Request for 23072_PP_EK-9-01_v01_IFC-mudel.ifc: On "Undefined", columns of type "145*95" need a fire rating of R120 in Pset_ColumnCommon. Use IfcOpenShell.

First a look at what the model holds.

```python
import ifcopenshell
import ifcopenshell.util.element

model = ifcopenshell.open("23072_PP_EK-9-01_v01_IFC-mudel.ifc")
print(model.schema)
storey = next(s for s in model.by_type("IfcBuildingStorey") if s.Name == "Undefined")
columns = [e for e in ifcopenshell.util.element.get_decomposition(storey) if e.is_a("IfcColumn")]
seen = {}
for e in columns:
    element_type = ifcopenshell.util.element.get_type(e)
    key = (element_type.Name if element_type != e and element_type else None, ifcopenshell.util.element.get_pset(e, "Pset_ColumnCommon", "FireRating"))
    seen[key] = seen.get(key, 0) + 1
for (name, value), count in sorted(seen.items(), key=str):
    print(count, "x", name, "|", value)
```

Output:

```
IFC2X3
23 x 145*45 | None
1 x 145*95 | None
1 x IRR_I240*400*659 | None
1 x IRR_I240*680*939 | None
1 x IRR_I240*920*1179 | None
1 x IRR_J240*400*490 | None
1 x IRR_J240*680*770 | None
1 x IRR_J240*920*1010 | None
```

```python
import ifcopenshell
import ifcopenshell.api.pset
import ifcopenshell.util.element

model = ifcopenshell.open("23072_PP_EK-9-01_v01_IFC-mudel.ifc")

storey = next(s for s in model.by_type("IfcBuildingStorey") if s.Name == "Undefined")
columns = [e for e in ifcopenshell.util.element.get_decomposition(storey) if e.is_a("IfcColumn")]

count = 0
for e in columns:
    element_type = ifcopenshell.util.element.get_type(e)
    if element_type in (None, e) or element_type.Name != "145*95":
        continue
    found = ifcopenshell.util.element.get_pset(e, "Pset_ColumnCommon", should_inherit=False)
    if found:
        pset = model.by_id(found["id"])
        if len(ifcopenshell.util.element.get_elements_by_pset(pset)) > 1:
            pset = ifcopenshell.api.pset.unshare_pset(model, products=[e], pset=pset)[0]
    else:
        pset = ifcopenshell.api.pset.add_pset(model, product=e, name="Pset_ColumnCommon")
    ifcopenshell.api.pset.edit_pset(model, pset=pset, properties={"FireRating": "R120"})
    count += 1

print(count, "columns updated")

model.write("23072_PP_EK-9-01_v01_IFC-mudel_edited.ifc")
```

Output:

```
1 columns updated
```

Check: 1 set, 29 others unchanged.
